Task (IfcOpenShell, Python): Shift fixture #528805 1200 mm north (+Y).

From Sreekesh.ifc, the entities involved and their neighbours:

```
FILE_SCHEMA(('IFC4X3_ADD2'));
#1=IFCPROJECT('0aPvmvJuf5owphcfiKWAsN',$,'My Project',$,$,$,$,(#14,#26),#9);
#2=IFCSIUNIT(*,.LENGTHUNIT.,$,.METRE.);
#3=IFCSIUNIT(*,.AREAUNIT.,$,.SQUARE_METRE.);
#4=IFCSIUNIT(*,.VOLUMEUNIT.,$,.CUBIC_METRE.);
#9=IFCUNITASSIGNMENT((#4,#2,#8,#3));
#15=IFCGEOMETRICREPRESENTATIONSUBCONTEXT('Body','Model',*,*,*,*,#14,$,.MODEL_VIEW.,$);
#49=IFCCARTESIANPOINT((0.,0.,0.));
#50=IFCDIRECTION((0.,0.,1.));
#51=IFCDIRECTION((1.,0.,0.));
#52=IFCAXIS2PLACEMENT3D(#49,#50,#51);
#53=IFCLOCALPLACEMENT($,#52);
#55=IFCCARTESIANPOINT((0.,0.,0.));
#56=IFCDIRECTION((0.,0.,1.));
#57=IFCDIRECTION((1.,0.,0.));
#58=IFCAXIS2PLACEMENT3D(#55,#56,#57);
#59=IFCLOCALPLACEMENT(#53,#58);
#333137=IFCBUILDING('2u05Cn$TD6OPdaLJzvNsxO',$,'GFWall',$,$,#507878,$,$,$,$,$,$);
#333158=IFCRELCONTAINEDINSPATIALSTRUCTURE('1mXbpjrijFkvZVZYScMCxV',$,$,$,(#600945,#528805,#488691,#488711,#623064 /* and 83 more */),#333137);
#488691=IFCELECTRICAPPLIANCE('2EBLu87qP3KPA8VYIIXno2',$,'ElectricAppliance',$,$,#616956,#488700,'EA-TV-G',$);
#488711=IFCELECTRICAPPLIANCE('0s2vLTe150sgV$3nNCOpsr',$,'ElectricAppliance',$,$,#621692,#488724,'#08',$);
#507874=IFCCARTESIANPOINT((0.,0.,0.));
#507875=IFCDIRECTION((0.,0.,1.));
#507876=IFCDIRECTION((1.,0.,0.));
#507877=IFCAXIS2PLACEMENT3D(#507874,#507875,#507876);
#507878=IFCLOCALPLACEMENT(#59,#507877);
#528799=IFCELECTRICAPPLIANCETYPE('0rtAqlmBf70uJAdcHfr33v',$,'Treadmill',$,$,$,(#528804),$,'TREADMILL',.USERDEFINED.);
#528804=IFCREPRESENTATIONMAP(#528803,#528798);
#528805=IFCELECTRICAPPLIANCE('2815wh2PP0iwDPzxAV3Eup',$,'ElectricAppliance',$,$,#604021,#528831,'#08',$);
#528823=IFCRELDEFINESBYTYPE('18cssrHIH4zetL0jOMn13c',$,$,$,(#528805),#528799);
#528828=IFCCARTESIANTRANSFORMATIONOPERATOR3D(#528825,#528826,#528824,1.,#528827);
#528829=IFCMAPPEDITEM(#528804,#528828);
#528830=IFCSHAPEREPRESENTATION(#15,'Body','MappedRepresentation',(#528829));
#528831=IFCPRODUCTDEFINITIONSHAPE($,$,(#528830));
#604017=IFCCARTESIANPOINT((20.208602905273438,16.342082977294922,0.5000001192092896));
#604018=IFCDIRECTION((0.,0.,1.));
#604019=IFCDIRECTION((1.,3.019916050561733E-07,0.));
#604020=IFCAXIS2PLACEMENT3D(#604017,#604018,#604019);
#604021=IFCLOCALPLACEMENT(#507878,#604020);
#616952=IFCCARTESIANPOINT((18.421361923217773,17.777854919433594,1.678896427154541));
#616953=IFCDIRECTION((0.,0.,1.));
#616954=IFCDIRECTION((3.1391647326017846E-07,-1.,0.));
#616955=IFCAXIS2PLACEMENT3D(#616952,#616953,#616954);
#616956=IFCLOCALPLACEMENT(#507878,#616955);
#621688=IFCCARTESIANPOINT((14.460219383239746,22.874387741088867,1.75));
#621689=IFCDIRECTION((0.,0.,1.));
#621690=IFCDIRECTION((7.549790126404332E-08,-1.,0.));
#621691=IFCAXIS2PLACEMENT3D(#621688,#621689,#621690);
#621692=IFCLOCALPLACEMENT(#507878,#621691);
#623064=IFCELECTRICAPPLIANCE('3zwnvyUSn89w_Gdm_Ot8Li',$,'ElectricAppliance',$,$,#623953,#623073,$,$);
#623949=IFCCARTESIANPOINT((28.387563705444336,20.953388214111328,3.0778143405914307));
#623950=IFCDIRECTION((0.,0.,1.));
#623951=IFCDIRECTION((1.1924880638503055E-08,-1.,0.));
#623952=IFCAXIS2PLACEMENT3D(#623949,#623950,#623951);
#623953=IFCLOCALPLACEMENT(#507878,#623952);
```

```python
import ifcopenshell
import ifcopenshell.api.geometry
import ifcopenshell.util.placement
import ifcopenshell.util.unit

model = ifcopenshell.open("Sreekesh.ifc")
unit_scale = ifcopenshell.util.unit.calculate_unit_scale(model)

item = model.by_guid("2815wh2PP0iwDPzxAV3Eup")
matrix = ifcopenshell.util.placement.get_local_placement(item.ObjectPlacement)
matrix[1, 3] += 1.2 / unit_scale
ifcopenshell.api.geometry.edit_object_placement(model, product=item, matrix=matrix, is_si=False)

print(ifcopenshell.util.placement.get_local_placement(item.ObjectPlacement).round(3) + 0.0)

model.write("Sreekesh_v2.ifc")
```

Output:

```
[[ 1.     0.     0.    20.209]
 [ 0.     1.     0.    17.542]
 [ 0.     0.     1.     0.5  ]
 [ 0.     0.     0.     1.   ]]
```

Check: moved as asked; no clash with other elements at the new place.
